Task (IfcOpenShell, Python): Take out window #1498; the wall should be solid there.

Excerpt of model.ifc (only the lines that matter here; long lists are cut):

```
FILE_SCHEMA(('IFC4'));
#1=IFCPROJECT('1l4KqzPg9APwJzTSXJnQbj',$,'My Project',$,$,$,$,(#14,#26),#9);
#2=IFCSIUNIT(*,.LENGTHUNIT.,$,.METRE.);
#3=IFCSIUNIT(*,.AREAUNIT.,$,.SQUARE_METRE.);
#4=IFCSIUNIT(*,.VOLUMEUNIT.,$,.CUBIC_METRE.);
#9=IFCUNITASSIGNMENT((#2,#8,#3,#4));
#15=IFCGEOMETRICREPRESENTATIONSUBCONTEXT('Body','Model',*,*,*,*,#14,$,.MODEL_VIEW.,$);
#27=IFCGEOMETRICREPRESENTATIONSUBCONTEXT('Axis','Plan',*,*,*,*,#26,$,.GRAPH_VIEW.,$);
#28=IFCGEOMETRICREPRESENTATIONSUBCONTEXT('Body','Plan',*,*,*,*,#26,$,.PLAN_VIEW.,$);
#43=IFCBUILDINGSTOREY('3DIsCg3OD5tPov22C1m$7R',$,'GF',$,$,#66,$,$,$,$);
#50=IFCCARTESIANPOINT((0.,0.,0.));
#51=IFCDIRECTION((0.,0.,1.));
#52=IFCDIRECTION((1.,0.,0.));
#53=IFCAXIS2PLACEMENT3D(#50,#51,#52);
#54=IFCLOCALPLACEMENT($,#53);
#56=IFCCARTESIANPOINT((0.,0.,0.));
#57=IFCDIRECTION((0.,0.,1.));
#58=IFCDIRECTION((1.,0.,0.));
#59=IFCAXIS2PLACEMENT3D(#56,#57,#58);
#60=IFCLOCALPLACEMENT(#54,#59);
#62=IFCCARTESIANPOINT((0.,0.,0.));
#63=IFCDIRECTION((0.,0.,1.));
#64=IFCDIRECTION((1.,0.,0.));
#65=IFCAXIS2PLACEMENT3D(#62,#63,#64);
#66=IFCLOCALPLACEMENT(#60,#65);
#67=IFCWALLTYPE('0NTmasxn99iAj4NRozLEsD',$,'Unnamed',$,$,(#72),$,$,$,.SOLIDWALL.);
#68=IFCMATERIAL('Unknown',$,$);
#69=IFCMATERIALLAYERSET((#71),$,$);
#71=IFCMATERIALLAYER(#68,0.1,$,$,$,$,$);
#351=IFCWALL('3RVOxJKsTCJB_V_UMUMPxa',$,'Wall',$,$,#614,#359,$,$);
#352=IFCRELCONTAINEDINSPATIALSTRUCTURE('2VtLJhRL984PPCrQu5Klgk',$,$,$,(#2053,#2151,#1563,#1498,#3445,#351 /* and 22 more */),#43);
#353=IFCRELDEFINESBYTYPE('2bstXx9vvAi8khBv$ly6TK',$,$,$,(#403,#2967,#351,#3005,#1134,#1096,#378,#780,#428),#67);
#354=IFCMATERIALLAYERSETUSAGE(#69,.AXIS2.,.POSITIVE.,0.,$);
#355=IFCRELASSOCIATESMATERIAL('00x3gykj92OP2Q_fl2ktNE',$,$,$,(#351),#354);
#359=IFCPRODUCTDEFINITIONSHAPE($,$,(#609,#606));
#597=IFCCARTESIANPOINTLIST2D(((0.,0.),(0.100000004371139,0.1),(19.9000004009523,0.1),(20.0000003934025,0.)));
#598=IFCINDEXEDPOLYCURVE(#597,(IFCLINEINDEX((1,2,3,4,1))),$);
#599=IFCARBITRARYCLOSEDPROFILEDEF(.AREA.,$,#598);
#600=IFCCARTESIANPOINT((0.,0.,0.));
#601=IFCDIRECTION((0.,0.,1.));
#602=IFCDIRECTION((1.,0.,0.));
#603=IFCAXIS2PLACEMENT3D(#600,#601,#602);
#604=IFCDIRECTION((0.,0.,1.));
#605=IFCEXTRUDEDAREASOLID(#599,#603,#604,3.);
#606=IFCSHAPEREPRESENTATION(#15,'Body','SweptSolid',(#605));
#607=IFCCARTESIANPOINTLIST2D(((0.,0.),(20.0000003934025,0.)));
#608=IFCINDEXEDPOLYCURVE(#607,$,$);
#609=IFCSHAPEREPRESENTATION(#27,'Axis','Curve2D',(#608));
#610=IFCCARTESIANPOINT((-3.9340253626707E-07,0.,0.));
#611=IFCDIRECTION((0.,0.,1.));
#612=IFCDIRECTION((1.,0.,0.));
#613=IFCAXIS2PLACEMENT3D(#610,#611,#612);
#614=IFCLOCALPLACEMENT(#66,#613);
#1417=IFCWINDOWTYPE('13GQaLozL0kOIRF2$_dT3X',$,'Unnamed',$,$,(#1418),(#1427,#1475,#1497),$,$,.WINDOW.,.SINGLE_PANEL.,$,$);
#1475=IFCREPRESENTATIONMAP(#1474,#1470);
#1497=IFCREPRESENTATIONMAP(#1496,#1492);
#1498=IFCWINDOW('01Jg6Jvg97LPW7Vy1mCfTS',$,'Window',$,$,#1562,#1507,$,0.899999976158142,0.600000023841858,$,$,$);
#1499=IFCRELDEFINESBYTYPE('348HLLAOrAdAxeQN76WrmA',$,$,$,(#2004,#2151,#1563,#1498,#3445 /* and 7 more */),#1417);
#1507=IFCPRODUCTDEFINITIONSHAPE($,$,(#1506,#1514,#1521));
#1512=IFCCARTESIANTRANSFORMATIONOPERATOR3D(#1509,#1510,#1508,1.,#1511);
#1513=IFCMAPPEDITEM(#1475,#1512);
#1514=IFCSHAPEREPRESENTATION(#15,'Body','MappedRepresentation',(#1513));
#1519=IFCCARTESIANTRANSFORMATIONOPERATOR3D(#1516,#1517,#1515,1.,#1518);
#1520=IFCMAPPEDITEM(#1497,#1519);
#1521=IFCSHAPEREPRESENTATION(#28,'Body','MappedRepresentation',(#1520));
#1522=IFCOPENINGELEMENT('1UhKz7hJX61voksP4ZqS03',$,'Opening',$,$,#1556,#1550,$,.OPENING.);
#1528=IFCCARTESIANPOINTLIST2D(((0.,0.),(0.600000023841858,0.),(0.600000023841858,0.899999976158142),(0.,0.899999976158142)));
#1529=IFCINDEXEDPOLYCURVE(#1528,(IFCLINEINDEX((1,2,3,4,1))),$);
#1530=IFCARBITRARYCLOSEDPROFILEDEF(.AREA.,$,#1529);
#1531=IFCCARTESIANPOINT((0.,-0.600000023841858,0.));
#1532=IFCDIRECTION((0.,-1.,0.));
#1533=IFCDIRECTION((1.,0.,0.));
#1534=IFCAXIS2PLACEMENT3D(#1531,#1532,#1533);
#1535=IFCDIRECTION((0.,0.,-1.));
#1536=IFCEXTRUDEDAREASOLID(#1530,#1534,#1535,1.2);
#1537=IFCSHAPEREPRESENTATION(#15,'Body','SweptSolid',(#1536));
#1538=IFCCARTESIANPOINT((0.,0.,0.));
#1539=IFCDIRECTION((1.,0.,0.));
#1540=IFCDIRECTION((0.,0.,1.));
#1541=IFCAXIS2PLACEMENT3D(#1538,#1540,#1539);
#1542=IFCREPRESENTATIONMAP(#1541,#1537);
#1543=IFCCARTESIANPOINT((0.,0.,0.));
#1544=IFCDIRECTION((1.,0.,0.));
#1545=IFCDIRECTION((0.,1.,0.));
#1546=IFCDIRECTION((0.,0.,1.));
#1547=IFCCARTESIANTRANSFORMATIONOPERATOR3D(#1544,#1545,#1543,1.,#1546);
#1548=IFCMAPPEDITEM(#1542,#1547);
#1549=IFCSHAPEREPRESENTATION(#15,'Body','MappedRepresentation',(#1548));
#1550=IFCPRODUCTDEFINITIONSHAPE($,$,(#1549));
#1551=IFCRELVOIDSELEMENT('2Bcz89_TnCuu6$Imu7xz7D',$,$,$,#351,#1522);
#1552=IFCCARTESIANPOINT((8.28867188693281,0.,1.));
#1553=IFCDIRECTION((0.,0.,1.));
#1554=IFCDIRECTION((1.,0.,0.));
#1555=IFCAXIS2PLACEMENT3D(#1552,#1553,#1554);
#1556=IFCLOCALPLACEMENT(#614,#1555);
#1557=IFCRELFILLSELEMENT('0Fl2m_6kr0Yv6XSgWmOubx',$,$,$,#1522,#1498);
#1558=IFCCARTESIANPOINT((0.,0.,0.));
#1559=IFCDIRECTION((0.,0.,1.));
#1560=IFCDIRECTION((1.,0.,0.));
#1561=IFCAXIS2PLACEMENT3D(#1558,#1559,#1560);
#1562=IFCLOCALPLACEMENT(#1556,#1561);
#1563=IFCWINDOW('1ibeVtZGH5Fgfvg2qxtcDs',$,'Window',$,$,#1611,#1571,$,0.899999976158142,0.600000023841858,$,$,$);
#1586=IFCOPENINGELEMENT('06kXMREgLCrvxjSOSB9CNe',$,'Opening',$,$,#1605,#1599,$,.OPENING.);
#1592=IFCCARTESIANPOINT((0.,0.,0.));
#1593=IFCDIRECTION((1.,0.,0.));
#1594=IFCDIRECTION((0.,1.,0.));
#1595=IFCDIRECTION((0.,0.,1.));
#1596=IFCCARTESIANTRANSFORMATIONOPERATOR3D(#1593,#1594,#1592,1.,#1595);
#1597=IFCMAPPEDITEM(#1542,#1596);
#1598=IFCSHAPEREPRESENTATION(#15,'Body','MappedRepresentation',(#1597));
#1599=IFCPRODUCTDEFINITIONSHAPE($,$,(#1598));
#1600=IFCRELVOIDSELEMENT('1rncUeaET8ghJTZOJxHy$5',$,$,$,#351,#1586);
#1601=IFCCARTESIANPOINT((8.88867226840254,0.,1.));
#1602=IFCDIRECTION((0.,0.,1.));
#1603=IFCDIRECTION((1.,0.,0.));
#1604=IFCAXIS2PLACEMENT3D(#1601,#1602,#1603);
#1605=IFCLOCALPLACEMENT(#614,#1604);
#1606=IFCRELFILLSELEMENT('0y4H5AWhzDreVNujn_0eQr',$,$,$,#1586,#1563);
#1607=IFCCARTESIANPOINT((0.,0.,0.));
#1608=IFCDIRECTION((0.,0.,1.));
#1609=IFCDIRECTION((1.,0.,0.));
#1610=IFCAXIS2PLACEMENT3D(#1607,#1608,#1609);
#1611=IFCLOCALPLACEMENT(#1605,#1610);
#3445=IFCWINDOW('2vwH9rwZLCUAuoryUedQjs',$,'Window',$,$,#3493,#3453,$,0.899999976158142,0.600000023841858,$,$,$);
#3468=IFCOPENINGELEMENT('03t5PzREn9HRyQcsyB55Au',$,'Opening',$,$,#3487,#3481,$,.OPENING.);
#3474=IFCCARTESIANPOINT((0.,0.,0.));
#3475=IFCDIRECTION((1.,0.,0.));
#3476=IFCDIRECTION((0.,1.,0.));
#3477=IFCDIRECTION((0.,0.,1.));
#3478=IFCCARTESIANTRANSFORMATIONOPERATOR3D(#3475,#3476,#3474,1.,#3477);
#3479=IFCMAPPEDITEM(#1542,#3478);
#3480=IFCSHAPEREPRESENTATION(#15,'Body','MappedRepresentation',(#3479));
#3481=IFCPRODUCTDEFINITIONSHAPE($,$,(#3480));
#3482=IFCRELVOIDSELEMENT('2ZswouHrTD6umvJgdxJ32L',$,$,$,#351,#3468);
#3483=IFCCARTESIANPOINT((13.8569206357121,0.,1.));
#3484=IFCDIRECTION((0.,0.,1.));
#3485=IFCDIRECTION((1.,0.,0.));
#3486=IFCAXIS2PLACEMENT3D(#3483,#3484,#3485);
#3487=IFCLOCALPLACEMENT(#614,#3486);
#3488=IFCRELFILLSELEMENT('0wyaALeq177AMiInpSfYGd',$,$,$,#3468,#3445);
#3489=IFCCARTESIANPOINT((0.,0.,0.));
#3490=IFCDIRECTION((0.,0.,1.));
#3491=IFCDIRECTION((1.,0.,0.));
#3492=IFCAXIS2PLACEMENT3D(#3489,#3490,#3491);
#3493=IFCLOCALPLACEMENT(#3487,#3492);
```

```python
import ifcopenshell
import ifcopenshell.api.feature
import ifcopenshell.api.root
import ifcopenshell.geom
import ifcopenshell.util.shape

model = ifcopenshell.open("model.ifc")
settings = ifcopenshell.geom.settings()


def volume(element):
    """Net volume in cubic metres, openings subtracted."""
    shape = ifcopenshell.geom.create_shape(settings, element)
    return ifcopenshell.util.shape.get_volume(shape.geometry)


window = model.by_id(1498)
opening = window.FillsVoids[0].RelatingOpeningElement
wall = opening.VoidsElements[0].RelatingBuildingElement
before = volume(wall)

ifcopenshell.api.root.remove_product(model, product=window)
ifcopenshell.api.feature.remove_feature(model, feature=opening)

after = volume(wall)

print(f"wall volume {before:.3f} -> {after:.3f} m3")

model.write("model_updated.ifc")
```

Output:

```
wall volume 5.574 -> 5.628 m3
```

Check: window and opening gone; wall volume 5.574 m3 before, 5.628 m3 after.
